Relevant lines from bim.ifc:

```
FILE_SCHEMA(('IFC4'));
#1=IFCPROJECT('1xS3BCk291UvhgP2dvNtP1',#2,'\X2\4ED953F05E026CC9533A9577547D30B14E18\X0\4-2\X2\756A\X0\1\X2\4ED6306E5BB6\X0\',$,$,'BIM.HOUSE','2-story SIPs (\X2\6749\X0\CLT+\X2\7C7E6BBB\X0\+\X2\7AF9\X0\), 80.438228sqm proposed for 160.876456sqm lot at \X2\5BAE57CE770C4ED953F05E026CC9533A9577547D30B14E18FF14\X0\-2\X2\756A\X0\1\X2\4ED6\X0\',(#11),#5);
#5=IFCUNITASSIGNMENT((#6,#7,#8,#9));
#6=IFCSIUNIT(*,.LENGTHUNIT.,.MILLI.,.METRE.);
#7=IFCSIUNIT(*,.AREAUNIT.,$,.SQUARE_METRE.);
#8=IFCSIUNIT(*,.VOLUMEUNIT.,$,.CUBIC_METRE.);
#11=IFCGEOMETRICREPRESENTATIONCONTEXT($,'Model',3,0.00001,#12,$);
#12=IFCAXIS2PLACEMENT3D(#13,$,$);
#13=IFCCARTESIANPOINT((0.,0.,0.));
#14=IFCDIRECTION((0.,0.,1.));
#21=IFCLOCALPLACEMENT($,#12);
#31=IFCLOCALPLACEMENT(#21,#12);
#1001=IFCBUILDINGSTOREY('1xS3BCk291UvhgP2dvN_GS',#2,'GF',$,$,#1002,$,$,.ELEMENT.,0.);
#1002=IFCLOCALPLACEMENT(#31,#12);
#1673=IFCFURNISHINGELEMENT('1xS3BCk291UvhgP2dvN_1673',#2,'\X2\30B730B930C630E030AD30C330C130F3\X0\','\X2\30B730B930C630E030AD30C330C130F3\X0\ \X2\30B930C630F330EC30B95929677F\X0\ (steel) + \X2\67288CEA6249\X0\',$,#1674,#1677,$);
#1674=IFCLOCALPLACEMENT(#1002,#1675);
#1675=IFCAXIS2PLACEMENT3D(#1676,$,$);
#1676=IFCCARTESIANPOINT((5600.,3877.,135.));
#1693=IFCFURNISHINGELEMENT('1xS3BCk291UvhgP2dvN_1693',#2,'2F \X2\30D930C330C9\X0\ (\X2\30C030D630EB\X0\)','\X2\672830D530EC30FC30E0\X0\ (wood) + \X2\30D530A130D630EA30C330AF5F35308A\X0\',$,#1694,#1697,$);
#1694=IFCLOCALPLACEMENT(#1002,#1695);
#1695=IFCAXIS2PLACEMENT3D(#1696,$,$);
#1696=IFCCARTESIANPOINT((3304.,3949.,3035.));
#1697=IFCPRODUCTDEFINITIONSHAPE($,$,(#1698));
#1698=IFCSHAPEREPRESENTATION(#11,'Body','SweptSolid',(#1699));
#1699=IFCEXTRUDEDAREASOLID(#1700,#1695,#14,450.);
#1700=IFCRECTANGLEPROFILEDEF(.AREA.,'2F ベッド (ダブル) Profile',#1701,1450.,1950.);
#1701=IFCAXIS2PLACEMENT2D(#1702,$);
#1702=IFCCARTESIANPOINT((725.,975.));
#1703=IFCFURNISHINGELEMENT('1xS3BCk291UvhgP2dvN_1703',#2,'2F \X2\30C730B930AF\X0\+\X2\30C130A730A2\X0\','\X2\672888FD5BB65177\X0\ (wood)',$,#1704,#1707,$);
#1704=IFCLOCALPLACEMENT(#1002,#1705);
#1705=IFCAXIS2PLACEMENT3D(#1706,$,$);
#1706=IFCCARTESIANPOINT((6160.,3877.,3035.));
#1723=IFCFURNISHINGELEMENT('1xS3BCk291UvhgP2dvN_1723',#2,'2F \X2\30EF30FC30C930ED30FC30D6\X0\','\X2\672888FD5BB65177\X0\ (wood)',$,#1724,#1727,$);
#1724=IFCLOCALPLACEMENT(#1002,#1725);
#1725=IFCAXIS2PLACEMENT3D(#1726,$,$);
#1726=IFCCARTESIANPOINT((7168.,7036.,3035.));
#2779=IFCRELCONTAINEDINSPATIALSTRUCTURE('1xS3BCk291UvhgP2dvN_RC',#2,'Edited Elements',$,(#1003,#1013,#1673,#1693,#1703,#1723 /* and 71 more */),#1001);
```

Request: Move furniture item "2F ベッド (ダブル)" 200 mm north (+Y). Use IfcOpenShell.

```python
import ifcopenshell
import ifcopenshell.api.geometry
import ifcopenshell.util.placement
import ifcopenshell.util.unit

model = ifcopenshell.open("bim.ifc")
unit_scale = ifcopenshell.util.unit.calculate_unit_scale(model)

item = model.by_guid("1xS3BCk291UvhgP2dvN_1693")
matrix = ifcopenshell.util.placement.get_local_placement(item.ObjectPlacement)
matrix[1, 3] += 0.2 / unit_scale
ifcopenshell.api.geometry.edit_object_placement(model, product=item, matrix=matrix, is_si=False)

print(ifcopenshell.util.placement.get_local_placement(item.ObjectPlacement).round(3) + 0.0)

model.write("bim_updated.ifc")
```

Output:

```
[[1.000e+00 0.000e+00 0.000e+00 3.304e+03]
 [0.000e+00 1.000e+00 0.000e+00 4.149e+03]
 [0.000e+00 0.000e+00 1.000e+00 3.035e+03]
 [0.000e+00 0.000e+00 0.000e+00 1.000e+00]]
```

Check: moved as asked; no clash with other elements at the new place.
